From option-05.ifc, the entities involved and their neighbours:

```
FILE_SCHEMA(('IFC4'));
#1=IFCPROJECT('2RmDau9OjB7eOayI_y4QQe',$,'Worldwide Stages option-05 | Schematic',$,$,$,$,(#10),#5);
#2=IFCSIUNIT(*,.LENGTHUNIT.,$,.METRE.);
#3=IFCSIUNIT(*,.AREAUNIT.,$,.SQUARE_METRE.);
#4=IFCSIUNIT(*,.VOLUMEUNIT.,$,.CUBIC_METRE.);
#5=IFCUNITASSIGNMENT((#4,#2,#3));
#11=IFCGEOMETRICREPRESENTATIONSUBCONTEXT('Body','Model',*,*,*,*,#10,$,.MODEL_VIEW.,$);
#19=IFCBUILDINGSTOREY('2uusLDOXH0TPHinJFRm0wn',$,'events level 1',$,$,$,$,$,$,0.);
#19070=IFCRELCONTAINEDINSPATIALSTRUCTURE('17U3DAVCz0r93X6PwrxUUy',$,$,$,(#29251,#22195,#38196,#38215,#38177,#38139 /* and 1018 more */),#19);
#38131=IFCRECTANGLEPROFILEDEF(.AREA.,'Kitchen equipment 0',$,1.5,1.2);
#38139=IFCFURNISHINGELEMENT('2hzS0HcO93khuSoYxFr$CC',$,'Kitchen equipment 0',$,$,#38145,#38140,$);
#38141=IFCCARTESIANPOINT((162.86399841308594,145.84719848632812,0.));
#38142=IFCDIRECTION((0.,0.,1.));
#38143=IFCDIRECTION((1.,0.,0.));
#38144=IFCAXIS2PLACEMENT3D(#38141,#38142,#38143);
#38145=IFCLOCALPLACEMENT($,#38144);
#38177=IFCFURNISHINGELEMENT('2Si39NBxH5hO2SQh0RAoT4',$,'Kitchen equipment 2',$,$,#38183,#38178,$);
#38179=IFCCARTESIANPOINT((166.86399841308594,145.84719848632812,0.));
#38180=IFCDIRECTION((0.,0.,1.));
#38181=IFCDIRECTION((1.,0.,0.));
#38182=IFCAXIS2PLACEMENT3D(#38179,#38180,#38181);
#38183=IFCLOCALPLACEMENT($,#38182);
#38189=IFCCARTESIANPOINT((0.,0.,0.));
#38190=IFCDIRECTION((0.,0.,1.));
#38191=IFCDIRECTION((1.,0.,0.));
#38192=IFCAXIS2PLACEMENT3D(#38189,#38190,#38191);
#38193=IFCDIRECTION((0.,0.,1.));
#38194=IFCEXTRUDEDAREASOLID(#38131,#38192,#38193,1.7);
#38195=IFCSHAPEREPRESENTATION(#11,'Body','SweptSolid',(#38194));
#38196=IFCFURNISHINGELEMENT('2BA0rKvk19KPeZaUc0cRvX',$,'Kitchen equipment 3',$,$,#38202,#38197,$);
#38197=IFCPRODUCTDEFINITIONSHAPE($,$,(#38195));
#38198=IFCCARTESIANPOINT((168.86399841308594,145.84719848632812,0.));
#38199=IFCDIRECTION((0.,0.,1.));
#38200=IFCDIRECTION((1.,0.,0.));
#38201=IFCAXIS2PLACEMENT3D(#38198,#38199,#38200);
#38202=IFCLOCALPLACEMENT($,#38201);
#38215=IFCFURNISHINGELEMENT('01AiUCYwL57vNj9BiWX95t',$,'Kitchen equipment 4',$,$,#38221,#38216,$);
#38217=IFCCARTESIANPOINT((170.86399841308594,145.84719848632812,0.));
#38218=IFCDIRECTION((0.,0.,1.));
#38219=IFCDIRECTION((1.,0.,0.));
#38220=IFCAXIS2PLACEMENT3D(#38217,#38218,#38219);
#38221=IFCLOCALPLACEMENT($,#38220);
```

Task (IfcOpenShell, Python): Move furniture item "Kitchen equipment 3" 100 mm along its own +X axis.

```python
import ifcopenshell
import ifcopenshell.api.geometry
import ifcopenshell.util.placement
import ifcopenshell.util.unit

model = ifcopenshell.open("option-05.ifc")
unit_scale = ifcopenshell.util.unit.calculate_unit_scale(model)

item = model.by_id(38196)
matrix = ifcopenshell.util.placement.get_local_placement(item.ObjectPlacement)
matrix[:3, 3] += matrix[:3, 0] * 0.1 / unit_scale
ifcopenshell.api.geometry.edit_object_placement(model, product=item, matrix=matrix, is_si=False)

print(ifcopenshell.util.placement.get_local_placement(item.ObjectPlacement).round(3) + 0.0)

model.write("option-05-out.ifc")
```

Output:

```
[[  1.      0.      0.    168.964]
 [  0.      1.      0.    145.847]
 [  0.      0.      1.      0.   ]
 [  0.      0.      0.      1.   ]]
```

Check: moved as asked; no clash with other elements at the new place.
